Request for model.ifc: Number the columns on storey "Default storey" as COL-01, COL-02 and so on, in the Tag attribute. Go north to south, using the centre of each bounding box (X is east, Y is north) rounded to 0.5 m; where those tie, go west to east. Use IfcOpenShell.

First a look at what the model holds.

```python
import ifcopenshell
import ifcopenshell.util.element
import ifcopenshell.util.placement

model = ifcopenshell.open("model.ifc")
print(model.schema)
storey = next(s for s in model.by_type("IfcBuildingStorey") if s.Name == "Default storey")
columns = [e for e in ifcopenshell.util.element.get_decomposition(storey) if e.is_a("IfcColumn")]
for e in sorted(columns, key=lambda e: e.id()):
    origin = ifcopenshell.util.placement.get_local_placement(e.ObjectPlacement)[:3, 3]
    print(e.id(), e.Tag, e.Name, origin.round(2) + 0.0, sep=" | ")
```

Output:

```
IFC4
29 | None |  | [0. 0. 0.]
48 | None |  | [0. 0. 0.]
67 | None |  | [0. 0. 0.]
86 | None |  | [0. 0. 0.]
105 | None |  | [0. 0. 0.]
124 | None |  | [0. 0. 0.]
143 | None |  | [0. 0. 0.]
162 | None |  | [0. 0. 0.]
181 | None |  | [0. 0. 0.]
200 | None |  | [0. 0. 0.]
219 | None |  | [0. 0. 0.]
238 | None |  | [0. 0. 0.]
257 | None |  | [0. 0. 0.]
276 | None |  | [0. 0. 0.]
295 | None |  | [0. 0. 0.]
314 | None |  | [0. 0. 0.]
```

```python
import ifcopenshell
import ifcopenshell.geom
import ifcopenshell.util.element
import ifcopenshell.util.shape

model = ifcopenshell.open("model.ifc")
settings = ifcopenshell.geom.settings()
settings.set("use-world-coords", True)


def centre(element):
    shape = ifcopenshell.geom.create_shape(settings, element)
    return ifcopenshell.util.shape.get_bbox_centroid(shape.geometry)


storey = next(s for s in model.by_type("IfcBuildingStorey") if s.Name == "Default storey")
columns = [e for e in ifcopenshell.util.element.get_decomposition(storey) if e.is_a("IfcColumn")]

# Insertion points can sit at a corner or the storey origin, so sort by the geometry (in metres).
centres = {e: centre(e) for e in columns}
columns.sort(key=lambda e: (-round(centres[e][1] / 0.5), centres[e][0]))

for i, e in enumerate(columns, start=1):
    number = f"COL-{i:02d}"
    e.Tag = number
    print(e.id(), number)

model.write("model_updated.ifc")
```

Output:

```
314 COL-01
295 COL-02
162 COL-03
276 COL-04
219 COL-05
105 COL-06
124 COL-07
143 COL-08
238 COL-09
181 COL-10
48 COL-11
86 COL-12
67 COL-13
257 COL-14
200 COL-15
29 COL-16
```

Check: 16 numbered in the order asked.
